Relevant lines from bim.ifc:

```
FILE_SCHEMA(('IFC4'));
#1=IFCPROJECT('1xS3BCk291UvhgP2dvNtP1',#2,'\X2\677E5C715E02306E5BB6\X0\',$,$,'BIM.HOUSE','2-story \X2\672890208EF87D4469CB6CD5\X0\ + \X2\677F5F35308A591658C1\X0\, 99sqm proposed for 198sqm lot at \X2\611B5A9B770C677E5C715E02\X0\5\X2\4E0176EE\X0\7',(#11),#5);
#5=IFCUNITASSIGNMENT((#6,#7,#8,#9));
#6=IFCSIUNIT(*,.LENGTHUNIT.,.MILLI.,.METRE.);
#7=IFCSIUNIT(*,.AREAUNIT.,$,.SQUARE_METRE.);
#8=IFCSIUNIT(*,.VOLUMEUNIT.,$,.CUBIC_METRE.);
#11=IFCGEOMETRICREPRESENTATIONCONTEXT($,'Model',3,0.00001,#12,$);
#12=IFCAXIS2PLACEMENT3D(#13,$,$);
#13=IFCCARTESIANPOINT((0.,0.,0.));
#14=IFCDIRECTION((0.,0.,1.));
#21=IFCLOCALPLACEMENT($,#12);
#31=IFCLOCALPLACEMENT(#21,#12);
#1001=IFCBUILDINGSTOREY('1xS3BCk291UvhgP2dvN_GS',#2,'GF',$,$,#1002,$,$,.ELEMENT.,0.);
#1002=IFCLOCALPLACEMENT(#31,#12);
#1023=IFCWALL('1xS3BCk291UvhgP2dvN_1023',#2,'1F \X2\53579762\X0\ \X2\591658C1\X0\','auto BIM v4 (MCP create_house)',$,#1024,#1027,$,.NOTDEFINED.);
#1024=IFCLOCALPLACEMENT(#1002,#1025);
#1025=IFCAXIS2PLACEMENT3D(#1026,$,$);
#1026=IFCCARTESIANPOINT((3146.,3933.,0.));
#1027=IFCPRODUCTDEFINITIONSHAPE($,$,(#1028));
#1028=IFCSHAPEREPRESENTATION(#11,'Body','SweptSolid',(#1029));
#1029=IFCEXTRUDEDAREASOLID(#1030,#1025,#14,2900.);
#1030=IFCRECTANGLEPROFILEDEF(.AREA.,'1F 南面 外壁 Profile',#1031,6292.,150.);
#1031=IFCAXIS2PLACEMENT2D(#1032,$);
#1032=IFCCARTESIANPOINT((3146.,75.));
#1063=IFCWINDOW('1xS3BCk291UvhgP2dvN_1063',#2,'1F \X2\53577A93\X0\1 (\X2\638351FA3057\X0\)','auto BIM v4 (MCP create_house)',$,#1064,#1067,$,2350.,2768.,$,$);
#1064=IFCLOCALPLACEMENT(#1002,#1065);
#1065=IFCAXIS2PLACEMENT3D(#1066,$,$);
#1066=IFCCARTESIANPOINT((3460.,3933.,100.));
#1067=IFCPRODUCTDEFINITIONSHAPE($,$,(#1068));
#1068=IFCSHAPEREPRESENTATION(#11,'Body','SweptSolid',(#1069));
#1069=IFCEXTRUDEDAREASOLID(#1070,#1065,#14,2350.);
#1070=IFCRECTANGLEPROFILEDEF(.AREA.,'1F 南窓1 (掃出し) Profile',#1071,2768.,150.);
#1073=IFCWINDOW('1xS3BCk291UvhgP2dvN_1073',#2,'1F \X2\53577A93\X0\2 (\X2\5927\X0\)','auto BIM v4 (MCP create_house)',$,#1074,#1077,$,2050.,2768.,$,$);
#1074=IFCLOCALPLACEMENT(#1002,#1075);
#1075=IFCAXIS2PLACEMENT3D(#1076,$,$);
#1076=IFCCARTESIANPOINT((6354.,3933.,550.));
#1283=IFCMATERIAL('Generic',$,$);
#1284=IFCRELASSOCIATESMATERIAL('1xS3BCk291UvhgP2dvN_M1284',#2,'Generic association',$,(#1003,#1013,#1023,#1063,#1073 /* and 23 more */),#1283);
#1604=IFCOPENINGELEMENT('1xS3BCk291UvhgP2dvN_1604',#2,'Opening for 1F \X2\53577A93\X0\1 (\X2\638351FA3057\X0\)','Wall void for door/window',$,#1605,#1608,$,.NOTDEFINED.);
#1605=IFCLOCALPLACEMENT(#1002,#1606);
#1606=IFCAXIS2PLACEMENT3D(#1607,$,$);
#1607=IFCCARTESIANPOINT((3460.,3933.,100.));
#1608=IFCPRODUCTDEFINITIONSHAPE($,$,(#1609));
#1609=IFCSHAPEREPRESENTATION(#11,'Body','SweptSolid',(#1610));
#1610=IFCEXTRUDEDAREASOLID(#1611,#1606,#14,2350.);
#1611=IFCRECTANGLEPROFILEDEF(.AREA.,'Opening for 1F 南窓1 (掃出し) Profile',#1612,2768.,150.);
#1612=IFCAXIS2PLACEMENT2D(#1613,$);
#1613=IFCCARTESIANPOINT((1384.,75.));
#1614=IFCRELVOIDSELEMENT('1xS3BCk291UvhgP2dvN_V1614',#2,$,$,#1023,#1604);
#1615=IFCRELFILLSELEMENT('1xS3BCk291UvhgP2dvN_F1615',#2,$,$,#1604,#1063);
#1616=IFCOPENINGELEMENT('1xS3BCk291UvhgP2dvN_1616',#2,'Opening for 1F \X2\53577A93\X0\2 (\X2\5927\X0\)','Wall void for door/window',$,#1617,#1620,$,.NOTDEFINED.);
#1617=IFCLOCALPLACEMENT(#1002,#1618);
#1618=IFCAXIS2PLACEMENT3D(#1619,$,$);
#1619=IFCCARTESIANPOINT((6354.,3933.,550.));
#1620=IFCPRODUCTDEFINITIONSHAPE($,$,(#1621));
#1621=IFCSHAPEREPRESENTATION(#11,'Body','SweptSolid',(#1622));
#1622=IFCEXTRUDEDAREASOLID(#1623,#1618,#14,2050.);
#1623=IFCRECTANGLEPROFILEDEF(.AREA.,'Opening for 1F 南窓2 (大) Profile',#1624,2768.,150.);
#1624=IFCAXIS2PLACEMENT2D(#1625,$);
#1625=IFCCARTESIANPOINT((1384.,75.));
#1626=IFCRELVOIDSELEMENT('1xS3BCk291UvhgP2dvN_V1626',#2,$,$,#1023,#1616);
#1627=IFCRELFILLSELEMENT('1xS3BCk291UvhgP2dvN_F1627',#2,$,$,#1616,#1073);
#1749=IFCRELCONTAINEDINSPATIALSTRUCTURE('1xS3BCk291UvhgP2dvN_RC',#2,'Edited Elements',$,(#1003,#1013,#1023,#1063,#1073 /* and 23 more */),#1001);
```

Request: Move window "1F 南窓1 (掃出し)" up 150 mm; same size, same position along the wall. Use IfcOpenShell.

```python
import numpy as np
import ifcopenshell
import ifcopenshell.api.geometry
import ifcopenshell.util.placement
import ifcopenshell.util.unit

model = ifcopenshell.open("bim.ifc")
unit_scale = ifcopenshell.util.unit.calculate_unit_scale(model)

window = model.by_guid("1xS3BCk291UvhgP2dvN_1063")
opening = window.FillsVoids[0].RelatingOpeningElement
dz = 150.0

shift = np.array([0.0, 0.0, dz])
# The window is not placed relative to its opening, so move both.
for product in (opening, window):
    matrix = ifcopenshell.util.placement.get_local_placement(product.ObjectPlacement)
    matrix[:3, 3] += shift
    ifcopenshell.api.geometry.edit_object_placement(model, product=product, matrix=matrix, is_si=False)

print(f"moved by {dz * unit_scale:+.3f} m")

model.write("bim_v2.ifc")
```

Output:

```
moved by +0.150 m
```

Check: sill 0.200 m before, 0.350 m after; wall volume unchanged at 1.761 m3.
